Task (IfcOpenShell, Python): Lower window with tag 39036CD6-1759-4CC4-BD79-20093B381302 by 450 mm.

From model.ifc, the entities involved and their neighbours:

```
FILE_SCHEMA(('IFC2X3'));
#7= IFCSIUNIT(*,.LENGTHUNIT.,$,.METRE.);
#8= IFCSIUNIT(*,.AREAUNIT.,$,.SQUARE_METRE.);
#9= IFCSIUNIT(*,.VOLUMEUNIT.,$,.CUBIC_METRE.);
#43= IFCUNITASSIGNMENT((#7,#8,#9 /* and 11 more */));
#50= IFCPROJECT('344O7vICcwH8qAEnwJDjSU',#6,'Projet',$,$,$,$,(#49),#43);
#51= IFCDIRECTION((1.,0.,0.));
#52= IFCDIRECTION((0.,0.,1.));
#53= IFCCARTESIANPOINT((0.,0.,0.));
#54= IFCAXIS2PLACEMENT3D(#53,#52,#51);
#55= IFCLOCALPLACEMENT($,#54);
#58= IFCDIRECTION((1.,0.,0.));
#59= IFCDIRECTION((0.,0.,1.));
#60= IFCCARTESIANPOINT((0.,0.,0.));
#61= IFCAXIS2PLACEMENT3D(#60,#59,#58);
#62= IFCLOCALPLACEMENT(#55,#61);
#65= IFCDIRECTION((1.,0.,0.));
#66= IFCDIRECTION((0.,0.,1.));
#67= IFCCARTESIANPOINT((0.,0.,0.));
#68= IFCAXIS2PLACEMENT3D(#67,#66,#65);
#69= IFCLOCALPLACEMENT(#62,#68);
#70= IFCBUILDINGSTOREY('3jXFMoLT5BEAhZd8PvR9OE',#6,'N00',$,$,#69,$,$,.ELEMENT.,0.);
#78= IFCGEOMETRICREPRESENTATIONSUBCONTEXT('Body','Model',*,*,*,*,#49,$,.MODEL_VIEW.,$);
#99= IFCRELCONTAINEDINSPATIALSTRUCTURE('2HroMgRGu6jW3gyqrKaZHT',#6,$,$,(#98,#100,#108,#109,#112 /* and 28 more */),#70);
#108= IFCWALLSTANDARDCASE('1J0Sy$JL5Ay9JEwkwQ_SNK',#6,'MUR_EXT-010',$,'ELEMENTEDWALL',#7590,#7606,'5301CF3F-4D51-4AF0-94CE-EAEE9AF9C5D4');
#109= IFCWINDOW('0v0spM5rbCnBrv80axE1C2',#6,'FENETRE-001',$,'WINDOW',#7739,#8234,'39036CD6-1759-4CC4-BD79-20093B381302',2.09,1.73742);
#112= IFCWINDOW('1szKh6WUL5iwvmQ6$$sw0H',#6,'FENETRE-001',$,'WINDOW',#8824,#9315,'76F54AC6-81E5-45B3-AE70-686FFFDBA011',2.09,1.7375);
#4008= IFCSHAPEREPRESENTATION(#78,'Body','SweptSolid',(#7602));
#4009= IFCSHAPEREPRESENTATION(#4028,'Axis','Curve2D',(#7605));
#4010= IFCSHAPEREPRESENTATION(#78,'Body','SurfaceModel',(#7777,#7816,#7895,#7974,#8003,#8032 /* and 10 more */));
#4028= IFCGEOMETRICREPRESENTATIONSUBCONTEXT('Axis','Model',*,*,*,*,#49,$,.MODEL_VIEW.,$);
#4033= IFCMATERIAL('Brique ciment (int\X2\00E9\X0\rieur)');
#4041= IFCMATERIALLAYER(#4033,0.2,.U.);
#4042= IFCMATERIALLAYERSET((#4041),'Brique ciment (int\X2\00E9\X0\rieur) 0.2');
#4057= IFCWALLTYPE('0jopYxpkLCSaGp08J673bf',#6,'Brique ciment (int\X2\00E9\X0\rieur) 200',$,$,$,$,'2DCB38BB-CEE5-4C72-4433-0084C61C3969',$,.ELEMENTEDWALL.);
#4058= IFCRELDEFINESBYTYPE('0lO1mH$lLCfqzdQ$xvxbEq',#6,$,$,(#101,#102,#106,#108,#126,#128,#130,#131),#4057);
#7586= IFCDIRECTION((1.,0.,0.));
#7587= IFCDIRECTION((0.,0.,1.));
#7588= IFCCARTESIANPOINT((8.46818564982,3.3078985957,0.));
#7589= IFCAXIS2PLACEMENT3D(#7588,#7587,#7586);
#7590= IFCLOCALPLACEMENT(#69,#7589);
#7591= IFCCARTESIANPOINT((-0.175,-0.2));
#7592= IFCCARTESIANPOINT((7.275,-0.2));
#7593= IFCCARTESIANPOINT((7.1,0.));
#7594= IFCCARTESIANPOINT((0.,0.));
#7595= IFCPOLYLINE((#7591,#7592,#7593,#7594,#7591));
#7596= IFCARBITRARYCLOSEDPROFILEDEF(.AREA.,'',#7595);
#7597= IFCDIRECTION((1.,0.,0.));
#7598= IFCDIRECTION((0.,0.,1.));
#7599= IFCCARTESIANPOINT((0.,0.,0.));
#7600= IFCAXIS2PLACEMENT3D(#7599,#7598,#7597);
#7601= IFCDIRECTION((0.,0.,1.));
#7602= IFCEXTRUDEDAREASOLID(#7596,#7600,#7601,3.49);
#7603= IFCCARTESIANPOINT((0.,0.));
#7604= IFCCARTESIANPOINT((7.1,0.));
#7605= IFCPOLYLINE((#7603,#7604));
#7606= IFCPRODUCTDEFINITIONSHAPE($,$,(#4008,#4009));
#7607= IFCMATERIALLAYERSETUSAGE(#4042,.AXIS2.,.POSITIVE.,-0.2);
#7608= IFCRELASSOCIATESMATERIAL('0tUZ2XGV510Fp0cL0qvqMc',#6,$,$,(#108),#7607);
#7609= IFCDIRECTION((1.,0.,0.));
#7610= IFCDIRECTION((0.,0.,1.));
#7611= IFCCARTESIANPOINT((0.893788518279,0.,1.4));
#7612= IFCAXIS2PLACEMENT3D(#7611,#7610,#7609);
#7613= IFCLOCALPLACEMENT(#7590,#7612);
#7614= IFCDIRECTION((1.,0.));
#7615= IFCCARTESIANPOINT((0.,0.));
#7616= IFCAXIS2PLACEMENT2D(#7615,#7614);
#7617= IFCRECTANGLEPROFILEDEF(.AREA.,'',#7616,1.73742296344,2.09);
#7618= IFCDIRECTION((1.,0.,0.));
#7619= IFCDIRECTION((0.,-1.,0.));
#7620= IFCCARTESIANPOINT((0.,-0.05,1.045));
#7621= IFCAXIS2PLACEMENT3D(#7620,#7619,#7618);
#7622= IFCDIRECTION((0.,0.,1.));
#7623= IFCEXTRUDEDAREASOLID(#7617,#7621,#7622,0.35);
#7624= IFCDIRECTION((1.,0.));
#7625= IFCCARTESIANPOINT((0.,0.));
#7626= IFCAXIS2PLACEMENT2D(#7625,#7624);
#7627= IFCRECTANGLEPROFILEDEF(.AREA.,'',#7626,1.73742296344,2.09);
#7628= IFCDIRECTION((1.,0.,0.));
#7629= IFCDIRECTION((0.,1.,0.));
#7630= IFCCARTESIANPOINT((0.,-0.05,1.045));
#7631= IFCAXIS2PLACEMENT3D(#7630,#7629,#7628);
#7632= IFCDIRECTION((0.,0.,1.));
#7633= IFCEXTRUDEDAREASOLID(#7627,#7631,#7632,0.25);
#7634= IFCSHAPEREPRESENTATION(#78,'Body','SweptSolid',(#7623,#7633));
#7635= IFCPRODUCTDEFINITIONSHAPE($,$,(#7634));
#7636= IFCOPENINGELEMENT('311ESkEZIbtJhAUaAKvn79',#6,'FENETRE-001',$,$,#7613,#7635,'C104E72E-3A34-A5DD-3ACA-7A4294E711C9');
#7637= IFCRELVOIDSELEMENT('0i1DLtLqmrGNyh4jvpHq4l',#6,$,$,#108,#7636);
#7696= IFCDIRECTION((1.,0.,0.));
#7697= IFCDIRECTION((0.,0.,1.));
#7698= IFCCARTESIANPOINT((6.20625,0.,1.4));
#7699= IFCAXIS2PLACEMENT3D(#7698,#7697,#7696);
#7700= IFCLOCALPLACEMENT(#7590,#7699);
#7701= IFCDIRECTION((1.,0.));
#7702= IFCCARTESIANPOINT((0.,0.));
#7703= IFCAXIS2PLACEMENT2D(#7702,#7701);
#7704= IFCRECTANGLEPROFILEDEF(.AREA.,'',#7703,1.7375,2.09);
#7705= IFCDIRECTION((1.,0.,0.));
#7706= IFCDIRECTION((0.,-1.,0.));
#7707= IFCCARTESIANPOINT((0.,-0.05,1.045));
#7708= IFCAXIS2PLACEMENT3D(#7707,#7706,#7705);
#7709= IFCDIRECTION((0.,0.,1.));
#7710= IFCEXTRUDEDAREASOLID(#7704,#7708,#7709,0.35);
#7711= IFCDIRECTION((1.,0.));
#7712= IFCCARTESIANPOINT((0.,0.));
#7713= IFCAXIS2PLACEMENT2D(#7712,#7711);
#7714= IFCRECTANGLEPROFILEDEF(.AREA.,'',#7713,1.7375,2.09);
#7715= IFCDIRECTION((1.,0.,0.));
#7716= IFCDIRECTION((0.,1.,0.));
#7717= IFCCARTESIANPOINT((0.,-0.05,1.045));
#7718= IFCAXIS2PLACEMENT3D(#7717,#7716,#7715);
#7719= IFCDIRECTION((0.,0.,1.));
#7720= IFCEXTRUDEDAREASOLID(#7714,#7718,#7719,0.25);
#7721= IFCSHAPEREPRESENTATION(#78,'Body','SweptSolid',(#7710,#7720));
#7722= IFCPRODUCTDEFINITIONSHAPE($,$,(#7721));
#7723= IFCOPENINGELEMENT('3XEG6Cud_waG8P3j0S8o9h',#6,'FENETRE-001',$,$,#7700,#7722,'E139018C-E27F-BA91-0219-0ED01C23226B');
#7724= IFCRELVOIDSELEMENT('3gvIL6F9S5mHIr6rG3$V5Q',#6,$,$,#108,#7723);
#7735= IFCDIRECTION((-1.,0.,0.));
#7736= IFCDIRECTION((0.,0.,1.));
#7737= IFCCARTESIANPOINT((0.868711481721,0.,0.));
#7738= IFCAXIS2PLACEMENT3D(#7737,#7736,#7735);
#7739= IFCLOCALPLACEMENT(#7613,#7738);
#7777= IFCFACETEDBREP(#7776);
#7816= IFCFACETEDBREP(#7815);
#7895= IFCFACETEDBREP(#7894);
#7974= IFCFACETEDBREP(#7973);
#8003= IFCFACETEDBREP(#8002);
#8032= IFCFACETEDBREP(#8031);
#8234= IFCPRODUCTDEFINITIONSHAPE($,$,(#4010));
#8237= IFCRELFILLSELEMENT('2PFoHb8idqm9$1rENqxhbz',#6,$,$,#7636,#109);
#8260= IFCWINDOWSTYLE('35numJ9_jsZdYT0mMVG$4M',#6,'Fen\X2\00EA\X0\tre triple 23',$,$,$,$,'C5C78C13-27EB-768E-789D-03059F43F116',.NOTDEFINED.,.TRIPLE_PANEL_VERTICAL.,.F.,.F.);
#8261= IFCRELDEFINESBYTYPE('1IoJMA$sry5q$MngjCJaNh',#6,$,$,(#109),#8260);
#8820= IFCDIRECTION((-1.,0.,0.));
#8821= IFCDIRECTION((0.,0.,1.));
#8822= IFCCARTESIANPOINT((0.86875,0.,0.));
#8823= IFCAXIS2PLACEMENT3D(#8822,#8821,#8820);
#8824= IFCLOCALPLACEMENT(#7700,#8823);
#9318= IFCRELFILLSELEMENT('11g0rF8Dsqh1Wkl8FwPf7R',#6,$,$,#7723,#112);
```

```python
import numpy as np
import ifcopenshell
import ifcopenshell.api.geometry
import ifcopenshell.util.placement
import ifcopenshell.util.unit

model = ifcopenshell.open("model.ifc")
unit_scale = ifcopenshell.util.unit.calculate_unit_scale(model)

window = model.by_id(109)
opening = window.FillsVoids[0].RelatingOpeningElement
dz = -0.45 / unit_scale

shift = np.array([0.0, 0.0, dz])
# The window is placed relative to its opening, so it follows when the opening moves.
matrix = ifcopenshell.util.placement.get_local_placement(opening.ObjectPlacement)
matrix[:3, 3] += shift
ifcopenshell.api.geometry.edit_object_placement(
    model, product=opening, matrix=matrix, is_si=False, should_transform_children=True
)

print(f"moved by {dz * unit_scale:+.3f} m")

model.write("model_edited.ifc")
```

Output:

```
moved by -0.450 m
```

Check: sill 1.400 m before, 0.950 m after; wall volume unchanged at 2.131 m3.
